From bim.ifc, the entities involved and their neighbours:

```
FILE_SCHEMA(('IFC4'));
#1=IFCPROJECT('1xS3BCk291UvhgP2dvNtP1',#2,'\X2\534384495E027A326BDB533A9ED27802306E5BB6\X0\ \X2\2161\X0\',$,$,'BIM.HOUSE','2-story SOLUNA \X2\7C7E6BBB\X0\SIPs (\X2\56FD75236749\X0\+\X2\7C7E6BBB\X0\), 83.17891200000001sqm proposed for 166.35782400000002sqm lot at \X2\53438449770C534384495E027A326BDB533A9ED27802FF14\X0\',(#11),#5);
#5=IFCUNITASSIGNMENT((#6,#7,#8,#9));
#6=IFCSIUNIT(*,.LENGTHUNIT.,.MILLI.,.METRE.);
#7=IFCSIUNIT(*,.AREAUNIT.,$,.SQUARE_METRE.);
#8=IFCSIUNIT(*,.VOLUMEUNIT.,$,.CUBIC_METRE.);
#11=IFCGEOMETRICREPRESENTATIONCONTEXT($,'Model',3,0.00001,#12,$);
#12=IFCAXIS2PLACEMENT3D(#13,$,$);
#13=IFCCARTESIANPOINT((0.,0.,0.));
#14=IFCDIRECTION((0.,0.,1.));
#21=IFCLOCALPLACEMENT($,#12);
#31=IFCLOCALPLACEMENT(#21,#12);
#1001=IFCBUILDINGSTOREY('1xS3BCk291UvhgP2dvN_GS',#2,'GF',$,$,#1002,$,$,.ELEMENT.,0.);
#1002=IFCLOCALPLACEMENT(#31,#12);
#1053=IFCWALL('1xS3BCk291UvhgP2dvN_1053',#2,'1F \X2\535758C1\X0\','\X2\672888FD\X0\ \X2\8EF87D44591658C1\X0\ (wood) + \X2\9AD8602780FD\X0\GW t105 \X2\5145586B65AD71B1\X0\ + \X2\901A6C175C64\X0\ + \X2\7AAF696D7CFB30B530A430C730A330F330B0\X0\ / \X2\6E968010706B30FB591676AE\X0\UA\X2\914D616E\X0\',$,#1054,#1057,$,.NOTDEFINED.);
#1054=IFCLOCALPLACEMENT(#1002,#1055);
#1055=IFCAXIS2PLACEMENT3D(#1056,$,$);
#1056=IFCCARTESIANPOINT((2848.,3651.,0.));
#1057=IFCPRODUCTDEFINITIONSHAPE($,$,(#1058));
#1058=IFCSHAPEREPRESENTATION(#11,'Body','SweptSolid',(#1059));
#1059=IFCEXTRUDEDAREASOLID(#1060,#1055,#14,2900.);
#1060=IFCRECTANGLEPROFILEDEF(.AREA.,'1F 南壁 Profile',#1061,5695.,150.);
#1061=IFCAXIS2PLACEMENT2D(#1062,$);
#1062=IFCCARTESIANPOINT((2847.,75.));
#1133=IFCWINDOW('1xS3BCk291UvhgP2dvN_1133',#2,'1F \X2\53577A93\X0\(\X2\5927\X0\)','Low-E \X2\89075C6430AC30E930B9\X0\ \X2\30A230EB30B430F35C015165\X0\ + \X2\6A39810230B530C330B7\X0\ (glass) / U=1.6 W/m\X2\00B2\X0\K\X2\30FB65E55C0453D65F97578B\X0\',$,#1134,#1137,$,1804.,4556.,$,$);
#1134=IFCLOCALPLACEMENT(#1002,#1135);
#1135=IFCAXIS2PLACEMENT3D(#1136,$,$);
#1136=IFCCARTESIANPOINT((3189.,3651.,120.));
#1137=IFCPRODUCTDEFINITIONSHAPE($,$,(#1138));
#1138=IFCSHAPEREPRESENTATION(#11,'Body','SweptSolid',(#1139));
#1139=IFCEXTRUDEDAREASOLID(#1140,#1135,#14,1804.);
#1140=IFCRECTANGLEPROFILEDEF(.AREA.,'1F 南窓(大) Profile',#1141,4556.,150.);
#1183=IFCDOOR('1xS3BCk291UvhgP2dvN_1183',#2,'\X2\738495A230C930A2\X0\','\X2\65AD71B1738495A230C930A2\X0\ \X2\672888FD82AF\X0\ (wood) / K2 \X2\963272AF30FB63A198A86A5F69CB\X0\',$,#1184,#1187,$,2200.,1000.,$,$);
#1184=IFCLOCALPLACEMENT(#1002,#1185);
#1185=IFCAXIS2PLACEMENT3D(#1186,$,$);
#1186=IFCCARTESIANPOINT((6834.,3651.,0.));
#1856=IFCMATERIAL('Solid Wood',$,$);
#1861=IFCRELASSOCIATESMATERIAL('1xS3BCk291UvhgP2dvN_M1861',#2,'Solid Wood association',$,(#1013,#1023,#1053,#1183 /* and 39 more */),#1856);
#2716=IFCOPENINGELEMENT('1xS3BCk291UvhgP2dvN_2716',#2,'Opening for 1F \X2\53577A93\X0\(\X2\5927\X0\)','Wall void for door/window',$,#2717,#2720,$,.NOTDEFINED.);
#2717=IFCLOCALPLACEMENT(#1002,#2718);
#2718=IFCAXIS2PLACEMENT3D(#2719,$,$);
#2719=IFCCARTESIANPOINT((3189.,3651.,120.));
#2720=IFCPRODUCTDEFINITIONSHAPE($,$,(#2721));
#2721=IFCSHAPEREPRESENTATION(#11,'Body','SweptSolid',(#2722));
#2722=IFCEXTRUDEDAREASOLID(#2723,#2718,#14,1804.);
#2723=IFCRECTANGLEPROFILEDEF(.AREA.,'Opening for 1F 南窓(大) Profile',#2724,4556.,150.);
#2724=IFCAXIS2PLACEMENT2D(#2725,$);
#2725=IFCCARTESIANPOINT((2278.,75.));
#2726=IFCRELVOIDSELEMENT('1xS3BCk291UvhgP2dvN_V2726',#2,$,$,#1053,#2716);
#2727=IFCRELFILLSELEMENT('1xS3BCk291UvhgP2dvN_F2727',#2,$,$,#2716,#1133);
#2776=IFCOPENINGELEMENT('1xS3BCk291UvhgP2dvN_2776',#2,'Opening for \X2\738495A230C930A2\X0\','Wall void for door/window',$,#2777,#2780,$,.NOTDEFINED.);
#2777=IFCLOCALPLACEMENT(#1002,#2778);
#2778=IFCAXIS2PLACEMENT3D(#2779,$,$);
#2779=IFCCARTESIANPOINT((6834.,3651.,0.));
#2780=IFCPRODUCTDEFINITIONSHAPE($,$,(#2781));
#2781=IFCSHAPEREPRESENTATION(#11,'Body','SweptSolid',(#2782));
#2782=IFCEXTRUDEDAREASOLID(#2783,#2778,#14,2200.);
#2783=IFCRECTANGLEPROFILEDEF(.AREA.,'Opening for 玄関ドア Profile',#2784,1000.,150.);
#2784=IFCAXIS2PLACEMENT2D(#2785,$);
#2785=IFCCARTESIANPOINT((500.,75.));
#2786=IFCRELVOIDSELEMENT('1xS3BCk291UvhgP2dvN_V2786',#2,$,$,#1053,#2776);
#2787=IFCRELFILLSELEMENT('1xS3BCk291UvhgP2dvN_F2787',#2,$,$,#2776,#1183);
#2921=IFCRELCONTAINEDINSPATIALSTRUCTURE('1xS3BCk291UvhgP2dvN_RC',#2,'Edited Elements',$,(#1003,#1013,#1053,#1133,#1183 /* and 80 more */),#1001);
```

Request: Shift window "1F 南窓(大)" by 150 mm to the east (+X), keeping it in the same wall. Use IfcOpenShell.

```python
import ifcopenshell
import ifcopenshell.api.geometry
import ifcopenshell.util.placement

model = ifcopenshell.open("bim.ifc")

window = model.by_guid("1xS3BCk291UvhgP2dvN_1133")
opening = window.FillsVoids[0].RelatingOpeningElement
wall = opening.VoidsElements[0].RelatingBuildingElement

wall_matrix = ifcopenshell.util.placement.get_local_placement(wall.ObjectPlacement)
shift = wall_matrix[:3, 0] * 150.0
before = ifcopenshell.util.placement.get_local_placement(window.ObjectPlacement)[:3, 3].copy()

# The window is not placed relative to its opening, so move both.
for product in (opening, window):
    matrix = ifcopenshell.util.placement.get_local_placement(product.ObjectPlacement)
    matrix[:3, 3] += shift
    ifcopenshell.api.geometry.edit_object_placement(model, product=product, matrix=matrix, is_si=False)

after = ifcopenshell.util.placement.get_local_placement(window.ObjectPlacement)[:3, 3]
print("window moved by", (after - before).round(3) + 0.0)

model.write("bim_updated.ifc")
```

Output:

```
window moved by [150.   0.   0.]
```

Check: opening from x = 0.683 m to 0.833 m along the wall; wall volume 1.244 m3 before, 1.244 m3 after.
